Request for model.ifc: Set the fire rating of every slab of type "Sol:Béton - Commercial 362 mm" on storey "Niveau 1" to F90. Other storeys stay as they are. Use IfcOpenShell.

First a look at what the model holds.

```python
import ifcopenshell
import ifcopenshell.util.element

model = ifcopenshell.open("model.ifc")
print(model.schema)
storey = next(s for s in model.by_type("IfcBuildingStorey") if s.Name == "Niveau 1")
slabs = [e for e in ifcopenshell.util.element.get_decomposition(storey) if e.is_a("IfcSlab")]
seen = {}
for e in slabs:
    element_type = ifcopenshell.util.element.get_type(e)
    key = (element_type.Name if element_type != e and element_type else None, ifcopenshell.util.element.get_pset(e, "Pset_SlabCommon", "FireRating"))
    seen[key] = seen.get(key, 0) + 1
for (name, value), count in sorted(seen.items(), key=str):
    print(count, "x", name, "|", value)
```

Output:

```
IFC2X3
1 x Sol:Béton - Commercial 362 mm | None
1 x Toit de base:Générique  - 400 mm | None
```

```python
import ifcopenshell
import ifcopenshell.api.pset
import ifcopenshell.util.element

model = ifcopenshell.open("model.ifc")

storey = next(s for s in model.by_type("IfcBuildingStorey") if s.Name == "Niveau 1")
slabs = [e for e in ifcopenshell.util.element.get_decomposition(storey) if e.is_a("IfcSlab")]

count = 0
for e in slabs:
    element_type = ifcopenshell.util.element.get_type(e)
    if element_type in (None, e) or element_type.Name != 'Sol:Béton - Commercial 362\xa0mm':
        continue
    # add_pset returns the element's existing set when there is one.
    pset = ifcopenshell.api.pset.add_pset(model, product=e, name="Pset_SlabCommon")
    ifcopenshell.api.pset.edit_pset(model, pset=pset, properties={"FireRating": "F90"})
    count += 1

print(count, "slabs updated")

model.write("model_v2.ifc")
```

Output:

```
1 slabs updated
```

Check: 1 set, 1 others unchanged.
